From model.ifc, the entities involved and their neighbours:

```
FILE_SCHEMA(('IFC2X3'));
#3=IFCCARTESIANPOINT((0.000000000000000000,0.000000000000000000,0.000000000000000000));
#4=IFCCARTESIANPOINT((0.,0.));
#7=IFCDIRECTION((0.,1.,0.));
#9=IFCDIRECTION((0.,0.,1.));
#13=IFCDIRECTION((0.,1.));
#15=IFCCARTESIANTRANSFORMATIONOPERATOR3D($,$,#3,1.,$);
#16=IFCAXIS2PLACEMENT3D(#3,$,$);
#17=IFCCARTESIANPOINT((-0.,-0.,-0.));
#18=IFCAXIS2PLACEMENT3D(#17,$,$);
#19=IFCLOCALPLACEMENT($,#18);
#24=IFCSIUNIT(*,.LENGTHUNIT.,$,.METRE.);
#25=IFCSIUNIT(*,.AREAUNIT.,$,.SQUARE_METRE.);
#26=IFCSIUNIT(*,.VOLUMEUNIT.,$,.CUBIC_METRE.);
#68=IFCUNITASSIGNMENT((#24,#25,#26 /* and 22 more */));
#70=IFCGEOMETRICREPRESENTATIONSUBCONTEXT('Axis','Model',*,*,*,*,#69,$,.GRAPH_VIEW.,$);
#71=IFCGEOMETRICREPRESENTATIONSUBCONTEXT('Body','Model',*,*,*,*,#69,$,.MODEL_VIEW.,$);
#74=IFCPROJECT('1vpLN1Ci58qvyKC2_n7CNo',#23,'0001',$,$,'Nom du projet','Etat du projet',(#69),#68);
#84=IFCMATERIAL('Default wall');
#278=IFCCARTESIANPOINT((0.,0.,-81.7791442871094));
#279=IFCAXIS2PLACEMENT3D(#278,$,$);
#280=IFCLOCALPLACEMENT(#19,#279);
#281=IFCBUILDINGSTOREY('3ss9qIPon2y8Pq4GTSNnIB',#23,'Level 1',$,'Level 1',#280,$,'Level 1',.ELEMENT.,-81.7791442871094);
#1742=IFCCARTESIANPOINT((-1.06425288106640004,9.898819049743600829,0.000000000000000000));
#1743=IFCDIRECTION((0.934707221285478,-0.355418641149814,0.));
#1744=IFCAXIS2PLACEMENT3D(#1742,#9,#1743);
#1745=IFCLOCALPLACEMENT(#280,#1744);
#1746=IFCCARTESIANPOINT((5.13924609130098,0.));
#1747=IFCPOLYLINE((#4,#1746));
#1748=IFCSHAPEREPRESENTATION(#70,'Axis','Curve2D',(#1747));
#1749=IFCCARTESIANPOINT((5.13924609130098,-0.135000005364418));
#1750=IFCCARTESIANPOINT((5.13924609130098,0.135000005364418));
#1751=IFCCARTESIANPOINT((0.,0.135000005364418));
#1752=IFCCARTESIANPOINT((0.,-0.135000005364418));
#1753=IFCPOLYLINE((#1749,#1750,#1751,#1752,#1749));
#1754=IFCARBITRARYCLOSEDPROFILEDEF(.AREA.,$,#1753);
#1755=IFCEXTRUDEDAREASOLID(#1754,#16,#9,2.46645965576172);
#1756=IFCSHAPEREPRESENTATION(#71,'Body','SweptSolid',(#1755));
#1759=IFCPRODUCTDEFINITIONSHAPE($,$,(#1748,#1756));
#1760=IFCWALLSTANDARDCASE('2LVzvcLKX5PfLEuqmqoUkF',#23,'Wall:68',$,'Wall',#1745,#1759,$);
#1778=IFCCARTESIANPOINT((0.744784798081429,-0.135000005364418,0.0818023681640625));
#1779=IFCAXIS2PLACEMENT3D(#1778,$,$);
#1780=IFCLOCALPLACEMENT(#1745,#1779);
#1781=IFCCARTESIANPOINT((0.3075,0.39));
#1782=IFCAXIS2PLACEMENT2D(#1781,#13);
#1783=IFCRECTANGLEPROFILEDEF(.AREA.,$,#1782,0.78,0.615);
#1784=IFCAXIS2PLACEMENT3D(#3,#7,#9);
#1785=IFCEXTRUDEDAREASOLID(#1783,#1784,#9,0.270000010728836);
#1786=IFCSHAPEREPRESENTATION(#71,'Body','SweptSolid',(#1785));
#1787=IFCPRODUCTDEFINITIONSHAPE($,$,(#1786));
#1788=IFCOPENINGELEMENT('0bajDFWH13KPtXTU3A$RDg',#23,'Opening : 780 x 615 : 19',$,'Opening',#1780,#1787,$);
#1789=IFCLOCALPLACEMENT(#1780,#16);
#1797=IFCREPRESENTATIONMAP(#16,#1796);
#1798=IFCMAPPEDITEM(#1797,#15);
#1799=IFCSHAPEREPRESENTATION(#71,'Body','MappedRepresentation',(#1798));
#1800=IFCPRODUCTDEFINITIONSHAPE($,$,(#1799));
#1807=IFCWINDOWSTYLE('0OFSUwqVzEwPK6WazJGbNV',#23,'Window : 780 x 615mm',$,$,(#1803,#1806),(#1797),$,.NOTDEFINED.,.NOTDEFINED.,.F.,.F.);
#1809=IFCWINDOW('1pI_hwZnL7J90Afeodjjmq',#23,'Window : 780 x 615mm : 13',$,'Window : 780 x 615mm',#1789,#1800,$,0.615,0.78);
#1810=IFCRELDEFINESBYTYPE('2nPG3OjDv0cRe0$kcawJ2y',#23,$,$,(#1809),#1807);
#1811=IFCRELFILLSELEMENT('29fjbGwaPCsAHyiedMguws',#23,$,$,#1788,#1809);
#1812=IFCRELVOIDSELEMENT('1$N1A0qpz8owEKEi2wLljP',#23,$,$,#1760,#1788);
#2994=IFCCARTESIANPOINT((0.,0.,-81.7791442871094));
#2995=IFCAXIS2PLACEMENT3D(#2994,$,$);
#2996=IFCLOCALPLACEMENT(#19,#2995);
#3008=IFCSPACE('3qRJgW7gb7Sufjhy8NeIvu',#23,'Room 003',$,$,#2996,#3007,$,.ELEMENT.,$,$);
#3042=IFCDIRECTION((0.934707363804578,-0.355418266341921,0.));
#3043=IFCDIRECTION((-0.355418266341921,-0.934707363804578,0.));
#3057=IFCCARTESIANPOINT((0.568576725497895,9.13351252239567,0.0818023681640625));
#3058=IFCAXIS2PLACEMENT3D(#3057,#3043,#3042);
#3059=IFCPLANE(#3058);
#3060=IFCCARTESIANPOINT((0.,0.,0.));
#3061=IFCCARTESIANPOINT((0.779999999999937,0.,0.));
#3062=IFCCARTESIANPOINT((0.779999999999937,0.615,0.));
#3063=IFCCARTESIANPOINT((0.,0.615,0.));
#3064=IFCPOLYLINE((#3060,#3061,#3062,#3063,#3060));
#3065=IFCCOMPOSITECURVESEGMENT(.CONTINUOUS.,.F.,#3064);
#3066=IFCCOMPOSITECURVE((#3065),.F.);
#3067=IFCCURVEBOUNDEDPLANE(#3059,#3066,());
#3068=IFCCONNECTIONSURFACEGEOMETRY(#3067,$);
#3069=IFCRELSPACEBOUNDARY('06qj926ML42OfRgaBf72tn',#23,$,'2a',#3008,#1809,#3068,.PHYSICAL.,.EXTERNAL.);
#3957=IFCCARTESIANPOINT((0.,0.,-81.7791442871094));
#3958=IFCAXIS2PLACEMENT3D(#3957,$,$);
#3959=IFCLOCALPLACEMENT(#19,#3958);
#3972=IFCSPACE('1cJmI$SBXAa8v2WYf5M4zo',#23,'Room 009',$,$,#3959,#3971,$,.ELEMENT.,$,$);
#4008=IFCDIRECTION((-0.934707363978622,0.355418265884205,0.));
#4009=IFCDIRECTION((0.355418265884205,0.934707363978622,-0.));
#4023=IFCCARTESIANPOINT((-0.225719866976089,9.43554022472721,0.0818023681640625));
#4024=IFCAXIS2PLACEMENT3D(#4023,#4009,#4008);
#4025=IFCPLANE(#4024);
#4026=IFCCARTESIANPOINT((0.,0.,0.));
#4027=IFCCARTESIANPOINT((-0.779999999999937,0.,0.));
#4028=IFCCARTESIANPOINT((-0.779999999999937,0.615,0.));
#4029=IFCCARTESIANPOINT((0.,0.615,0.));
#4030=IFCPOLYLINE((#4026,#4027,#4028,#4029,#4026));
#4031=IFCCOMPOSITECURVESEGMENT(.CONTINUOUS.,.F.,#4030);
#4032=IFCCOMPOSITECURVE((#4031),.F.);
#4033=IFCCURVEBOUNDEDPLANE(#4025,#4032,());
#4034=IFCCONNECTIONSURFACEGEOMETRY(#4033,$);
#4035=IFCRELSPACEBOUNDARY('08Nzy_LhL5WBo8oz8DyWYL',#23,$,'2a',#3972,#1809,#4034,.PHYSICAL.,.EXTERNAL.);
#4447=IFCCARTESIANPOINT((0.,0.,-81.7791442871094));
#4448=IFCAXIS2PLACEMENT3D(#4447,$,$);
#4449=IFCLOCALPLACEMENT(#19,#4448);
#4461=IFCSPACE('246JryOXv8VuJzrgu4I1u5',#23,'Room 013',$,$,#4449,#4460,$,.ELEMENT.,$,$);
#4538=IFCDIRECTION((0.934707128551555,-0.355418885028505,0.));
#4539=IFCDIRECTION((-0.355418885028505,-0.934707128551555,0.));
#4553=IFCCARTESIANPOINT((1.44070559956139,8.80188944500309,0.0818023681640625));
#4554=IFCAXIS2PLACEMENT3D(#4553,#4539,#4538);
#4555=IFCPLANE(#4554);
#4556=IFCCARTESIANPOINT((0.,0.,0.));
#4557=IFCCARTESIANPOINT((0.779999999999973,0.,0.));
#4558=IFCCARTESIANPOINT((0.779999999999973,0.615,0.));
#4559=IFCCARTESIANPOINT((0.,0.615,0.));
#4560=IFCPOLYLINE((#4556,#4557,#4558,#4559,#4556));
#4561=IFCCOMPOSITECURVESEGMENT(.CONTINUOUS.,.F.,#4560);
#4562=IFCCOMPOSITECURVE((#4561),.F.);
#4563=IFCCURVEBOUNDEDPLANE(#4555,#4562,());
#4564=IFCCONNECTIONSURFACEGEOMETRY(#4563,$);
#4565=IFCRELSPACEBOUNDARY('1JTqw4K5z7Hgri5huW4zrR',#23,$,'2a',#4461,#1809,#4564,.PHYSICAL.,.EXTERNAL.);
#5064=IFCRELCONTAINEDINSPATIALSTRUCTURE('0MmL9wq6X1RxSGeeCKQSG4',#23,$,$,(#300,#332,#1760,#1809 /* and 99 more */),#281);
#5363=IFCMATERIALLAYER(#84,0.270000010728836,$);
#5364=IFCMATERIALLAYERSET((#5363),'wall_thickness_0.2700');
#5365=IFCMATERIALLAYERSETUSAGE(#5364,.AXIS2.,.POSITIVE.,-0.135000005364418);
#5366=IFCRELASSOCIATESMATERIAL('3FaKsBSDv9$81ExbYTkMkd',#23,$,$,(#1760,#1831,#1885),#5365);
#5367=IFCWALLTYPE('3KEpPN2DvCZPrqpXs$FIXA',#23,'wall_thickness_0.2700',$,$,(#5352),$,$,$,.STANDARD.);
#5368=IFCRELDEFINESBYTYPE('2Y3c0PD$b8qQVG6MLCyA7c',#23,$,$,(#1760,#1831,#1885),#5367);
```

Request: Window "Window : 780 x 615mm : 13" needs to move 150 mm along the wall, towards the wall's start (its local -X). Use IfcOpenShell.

```python
import numpy as np
import ifcopenshell
import ifcopenshell.api.geometry
import ifcopenshell.util.placement

model = ifcopenshell.open("model.ifc")

window = model.by_guid("1pI_hwZnL7J90Afeodjjmq")
opening = window.FillsVoids[0].RelatingOpeningElement
wall = opening.VoidsElements[0].RelatingBuildingElement

wall_matrix = ifcopenshell.util.placement.get_local_placement(wall.ObjectPlacement)
shift = wall_matrix[:3, 0] * -0.15
before = ifcopenshell.util.placement.get_local_placement(window.ObjectPlacement)[:3, 3].copy()

# The window is placed relative to its opening, so it follows when the opening moves.
matrix = ifcopenshell.util.placement.get_local_placement(opening.ObjectPlacement)
matrix[:3, 3] += shift
ifcopenshell.api.geometry.edit_object_placement(
    model, product=opening, matrix=matrix, is_si=False, should_transform_children=True
)

# Space boundary surfaces are stored in each space's coordinates; move them too.
for rel in window.ProvidesBoundaries:
    if not rel.ConnectionGeometry:
        continue
    surface = rel.ConnectionGeometry.SurfaceOnRelatingElement.BasisSurface
    space_matrix = ifcopenshell.util.placement.get_local_placement(rel.RelatingSpace.ObjectPlacement)
    point = np.array(surface.Position.Location.Coordinates) + space_matrix[:3, :3].T @ shift
    surface.Position = model.createIfcAxis2Placement3D(
        model.createIfcCartesianPoint(point.tolist()), surface.Position.Axis, surface.Position.RefDirection
    )

after = ifcopenshell.util.placement.get_local_placement(window.ObjectPlacement)[:3, 3]
print("window moved by", (after - before).round(3) + 0.0)

model.write("model_v2.ifc")
```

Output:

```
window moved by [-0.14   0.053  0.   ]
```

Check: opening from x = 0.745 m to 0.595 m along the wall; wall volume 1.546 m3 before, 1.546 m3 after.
